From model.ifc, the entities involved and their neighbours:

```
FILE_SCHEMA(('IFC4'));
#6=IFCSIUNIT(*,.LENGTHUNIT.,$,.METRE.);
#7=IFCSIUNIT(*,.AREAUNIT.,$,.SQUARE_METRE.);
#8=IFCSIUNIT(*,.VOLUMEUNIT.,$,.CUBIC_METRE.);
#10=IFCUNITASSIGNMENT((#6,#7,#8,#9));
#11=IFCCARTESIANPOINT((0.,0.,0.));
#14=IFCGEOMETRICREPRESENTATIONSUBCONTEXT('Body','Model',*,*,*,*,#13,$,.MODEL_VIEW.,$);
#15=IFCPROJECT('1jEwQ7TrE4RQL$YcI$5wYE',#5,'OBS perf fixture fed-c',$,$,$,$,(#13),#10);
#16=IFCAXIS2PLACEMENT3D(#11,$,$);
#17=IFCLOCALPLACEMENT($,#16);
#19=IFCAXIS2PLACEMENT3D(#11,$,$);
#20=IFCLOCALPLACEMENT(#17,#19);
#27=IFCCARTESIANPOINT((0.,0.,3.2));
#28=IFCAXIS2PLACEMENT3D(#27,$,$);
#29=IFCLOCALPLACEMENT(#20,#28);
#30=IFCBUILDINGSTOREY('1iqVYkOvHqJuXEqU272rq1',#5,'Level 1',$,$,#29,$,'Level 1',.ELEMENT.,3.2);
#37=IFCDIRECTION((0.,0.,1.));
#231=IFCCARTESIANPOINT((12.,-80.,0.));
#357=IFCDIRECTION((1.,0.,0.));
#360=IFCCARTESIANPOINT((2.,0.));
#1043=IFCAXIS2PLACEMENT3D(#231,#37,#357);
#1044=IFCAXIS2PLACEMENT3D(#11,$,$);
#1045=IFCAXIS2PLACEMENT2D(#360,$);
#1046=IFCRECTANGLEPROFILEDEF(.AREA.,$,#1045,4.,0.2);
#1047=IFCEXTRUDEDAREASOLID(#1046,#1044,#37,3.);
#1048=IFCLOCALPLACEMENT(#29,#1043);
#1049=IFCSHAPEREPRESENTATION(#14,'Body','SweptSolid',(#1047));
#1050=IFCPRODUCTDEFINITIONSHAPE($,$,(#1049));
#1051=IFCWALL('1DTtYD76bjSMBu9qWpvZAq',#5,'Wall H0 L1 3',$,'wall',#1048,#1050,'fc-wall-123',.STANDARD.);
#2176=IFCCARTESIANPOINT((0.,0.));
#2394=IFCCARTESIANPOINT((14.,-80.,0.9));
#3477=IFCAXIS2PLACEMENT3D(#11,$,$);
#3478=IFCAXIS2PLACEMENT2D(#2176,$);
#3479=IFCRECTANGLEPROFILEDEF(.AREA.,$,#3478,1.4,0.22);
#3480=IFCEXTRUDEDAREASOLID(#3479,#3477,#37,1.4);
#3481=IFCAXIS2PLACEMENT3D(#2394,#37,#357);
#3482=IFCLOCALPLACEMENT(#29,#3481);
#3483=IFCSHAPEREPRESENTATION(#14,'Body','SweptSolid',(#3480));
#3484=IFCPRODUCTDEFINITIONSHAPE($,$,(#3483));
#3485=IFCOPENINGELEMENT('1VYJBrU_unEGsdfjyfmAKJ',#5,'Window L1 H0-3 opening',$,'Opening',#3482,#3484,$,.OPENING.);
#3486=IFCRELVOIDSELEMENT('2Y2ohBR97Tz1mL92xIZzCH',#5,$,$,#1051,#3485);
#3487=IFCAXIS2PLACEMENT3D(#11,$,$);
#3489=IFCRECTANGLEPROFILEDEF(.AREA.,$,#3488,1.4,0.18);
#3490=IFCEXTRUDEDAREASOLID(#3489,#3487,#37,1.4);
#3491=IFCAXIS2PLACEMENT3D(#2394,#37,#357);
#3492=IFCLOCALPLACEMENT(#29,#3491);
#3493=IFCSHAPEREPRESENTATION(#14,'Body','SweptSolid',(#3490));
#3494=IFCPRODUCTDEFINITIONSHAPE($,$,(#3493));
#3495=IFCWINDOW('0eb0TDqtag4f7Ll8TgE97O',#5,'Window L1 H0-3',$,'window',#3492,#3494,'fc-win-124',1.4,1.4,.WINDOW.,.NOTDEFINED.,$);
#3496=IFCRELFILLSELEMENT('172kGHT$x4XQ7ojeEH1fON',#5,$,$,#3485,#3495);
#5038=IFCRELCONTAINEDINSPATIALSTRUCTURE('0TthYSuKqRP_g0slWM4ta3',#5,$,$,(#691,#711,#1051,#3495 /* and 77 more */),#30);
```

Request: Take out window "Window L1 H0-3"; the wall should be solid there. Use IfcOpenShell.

```python
import ifcopenshell
import ifcopenshell.api.feature
import ifcopenshell.api.root
import ifcopenshell.geom
import ifcopenshell.util.shape

model = ifcopenshell.open("model.ifc")
settings = ifcopenshell.geom.settings()


def volume(element):
    """Net volume in cubic metres, openings subtracted."""
    shape = ifcopenshell.geom.create_shape(settings, element)
    return ifcopenshell.util.shape.get_volume(shape.geometry)


window = model.by_guid("0eb0TDqtag4f7Ll8TgE97O")
opening = window.FillsVoids[0].RelatingOpeningElement
wall = opening.VoidsElements[0].RelatingBuildingElement
before = volume(wall)

ifcopenshell.api.root.remove_product(model, product=window)
ifcopenshell.api.feature.remove_feature(model, feature=opening)

after = volume(wall)

print(f"wall volume {before:.3f} -> {after:.3f} m3")

model.write("model_edited.ifc")
```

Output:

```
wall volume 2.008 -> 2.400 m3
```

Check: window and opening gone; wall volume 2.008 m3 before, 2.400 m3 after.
